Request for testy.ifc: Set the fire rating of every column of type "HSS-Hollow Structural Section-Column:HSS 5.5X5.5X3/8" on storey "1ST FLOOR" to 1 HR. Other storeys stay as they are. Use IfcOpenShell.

First a look at what the model holds.

```python
import ifcopenshell
import ifcopenshell.util.element

model = ifcopenshell.open("testy.ifc")
print(model.schema)
storey = next(s for s in model.by_type("IfcBuildingStorey") if s.Name == "1ST FLOOR")
columns = [e for e in ifcopenshell.util.element.get_decomposition(storey) if e.is_a("IfcColumn")]
seen = {}
for e in columns:
    element_type = ifcopenshell.util.element.get_type(e)
    key = (element_type.Name if element_type != e and element_type else None, ifcopenshell.util.element.get_pset(e, "Pset_ColumnCommon", "FireRating"))
    seen[key] = seen.get(key, 0) + 1
for (name, value), count in sorted(seen.items(), key=str):
    print(count, "x", name, "|", value)
```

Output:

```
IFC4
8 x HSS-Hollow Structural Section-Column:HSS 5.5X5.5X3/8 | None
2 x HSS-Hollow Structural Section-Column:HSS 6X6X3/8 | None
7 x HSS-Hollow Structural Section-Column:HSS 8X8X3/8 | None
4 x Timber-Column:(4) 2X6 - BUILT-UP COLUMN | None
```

```python
import ifcopenshell
import ifcopenshell.api.pset
import ifcopenshell.util.element

model = ifcopenshell.open("testy.ifc")

storey = next(s for s in model.by_type("IfcBuildingStorey") if s.Name == "1ST FLOOR")
columns = [e for e in ifcopenshell.util.element.get_decomposition(storey) if e.is_a("IfcColumn")]

count = 0
for e in columns:
    element_type = ifcopenshell.util.element.get_type(e)
    if element_type in (None, e) or element_type.Name != "HSS-Hollow Structural Section-Column:HSS 5.5X5.5X3/8":
        continue
    # add_pset returns the element's existing set when there is one.
    pset = ifcopenshell.api.pset.add_pset(model, product=e, name="Pset_ColumnCommon")
    ifcopenshell.api.pset.edit_pset(model, pset=pset, properties={"FireRating": "1 HR"})
    count += 1

print(count, "columns updated")

model.write("testy_edited.ifc")
```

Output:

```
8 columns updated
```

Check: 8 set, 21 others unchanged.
